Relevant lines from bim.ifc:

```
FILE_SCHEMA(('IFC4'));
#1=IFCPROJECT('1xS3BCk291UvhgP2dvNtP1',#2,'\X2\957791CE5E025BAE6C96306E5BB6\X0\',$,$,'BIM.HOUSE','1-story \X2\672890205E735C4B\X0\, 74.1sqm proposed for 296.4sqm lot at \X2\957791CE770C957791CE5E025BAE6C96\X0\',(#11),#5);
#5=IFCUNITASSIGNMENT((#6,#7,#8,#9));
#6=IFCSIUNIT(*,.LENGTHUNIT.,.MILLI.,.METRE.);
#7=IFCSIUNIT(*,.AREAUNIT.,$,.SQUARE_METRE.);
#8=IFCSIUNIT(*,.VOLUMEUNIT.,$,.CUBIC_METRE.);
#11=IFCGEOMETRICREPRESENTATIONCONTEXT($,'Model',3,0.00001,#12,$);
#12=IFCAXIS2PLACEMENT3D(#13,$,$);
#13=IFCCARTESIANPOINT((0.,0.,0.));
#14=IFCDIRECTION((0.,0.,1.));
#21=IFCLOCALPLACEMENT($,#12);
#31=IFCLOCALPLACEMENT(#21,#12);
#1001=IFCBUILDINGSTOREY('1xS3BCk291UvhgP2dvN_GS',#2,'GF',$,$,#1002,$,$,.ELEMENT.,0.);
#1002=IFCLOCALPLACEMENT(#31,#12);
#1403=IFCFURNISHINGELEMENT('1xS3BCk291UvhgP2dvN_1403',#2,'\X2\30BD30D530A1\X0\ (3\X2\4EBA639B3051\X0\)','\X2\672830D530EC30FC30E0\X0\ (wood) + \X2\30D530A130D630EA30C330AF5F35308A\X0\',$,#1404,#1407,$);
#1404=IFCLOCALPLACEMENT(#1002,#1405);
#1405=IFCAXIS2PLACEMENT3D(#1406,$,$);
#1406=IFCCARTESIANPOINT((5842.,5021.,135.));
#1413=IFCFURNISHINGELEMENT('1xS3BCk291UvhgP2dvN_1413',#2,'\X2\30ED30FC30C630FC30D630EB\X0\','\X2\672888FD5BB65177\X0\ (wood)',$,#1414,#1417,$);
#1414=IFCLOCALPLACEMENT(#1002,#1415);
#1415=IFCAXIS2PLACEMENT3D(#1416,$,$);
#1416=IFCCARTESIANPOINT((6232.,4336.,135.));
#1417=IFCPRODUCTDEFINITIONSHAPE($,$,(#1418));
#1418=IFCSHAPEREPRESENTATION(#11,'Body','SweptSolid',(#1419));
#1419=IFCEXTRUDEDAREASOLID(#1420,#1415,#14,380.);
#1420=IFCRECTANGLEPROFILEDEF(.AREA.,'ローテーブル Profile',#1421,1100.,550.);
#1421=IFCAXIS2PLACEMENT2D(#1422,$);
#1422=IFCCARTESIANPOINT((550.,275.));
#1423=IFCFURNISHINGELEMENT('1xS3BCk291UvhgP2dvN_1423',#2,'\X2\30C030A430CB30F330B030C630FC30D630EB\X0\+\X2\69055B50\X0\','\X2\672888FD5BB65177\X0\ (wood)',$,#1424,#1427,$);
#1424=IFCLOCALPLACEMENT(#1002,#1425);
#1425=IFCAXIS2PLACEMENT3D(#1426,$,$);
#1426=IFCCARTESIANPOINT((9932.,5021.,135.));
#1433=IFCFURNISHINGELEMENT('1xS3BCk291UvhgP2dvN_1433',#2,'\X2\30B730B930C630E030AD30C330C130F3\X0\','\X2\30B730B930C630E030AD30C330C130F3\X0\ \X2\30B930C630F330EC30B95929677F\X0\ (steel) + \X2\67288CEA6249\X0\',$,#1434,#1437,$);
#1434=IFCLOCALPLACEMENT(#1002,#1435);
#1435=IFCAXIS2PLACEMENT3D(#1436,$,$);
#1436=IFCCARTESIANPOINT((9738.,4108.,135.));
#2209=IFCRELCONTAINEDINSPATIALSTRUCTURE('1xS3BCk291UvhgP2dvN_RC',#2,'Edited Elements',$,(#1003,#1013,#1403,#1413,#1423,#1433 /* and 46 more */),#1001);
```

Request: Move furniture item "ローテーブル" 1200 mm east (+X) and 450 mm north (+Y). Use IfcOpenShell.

```python
import ifcopenshell
import ifcopenshell.api.geometry
import ifcopenshell.util.placement
import ifcopenshell.util.unit

model = ifcopenshell.open("bim.ifc")
unit_scale = ifcopenshell.util.unit.calculate_unit_scale(model)

item = model.by_guid("1xS3BCk291UvhgP2dvN_1413")
matrix = ifcopenshell.util.placement.get_local_placement(item.ObjectPlacement)
matrix[0, 3] += 1.2 / unit_scale
matrix[1, 3] += 0.45 / unit_scale
ifcopenshell.api.geometry.edit_object_placement(model, product=item, matrix=matrix, is_si=False)

print(ifcopenshell.util.placement.get_local_placement(item.ObjectPlacement).round(3) + 0.0)

model.write("bim_edited.ifc")
```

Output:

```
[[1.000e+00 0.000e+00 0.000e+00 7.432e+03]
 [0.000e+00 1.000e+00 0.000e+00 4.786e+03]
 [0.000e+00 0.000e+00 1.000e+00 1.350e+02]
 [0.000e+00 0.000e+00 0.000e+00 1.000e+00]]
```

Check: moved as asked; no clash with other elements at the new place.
